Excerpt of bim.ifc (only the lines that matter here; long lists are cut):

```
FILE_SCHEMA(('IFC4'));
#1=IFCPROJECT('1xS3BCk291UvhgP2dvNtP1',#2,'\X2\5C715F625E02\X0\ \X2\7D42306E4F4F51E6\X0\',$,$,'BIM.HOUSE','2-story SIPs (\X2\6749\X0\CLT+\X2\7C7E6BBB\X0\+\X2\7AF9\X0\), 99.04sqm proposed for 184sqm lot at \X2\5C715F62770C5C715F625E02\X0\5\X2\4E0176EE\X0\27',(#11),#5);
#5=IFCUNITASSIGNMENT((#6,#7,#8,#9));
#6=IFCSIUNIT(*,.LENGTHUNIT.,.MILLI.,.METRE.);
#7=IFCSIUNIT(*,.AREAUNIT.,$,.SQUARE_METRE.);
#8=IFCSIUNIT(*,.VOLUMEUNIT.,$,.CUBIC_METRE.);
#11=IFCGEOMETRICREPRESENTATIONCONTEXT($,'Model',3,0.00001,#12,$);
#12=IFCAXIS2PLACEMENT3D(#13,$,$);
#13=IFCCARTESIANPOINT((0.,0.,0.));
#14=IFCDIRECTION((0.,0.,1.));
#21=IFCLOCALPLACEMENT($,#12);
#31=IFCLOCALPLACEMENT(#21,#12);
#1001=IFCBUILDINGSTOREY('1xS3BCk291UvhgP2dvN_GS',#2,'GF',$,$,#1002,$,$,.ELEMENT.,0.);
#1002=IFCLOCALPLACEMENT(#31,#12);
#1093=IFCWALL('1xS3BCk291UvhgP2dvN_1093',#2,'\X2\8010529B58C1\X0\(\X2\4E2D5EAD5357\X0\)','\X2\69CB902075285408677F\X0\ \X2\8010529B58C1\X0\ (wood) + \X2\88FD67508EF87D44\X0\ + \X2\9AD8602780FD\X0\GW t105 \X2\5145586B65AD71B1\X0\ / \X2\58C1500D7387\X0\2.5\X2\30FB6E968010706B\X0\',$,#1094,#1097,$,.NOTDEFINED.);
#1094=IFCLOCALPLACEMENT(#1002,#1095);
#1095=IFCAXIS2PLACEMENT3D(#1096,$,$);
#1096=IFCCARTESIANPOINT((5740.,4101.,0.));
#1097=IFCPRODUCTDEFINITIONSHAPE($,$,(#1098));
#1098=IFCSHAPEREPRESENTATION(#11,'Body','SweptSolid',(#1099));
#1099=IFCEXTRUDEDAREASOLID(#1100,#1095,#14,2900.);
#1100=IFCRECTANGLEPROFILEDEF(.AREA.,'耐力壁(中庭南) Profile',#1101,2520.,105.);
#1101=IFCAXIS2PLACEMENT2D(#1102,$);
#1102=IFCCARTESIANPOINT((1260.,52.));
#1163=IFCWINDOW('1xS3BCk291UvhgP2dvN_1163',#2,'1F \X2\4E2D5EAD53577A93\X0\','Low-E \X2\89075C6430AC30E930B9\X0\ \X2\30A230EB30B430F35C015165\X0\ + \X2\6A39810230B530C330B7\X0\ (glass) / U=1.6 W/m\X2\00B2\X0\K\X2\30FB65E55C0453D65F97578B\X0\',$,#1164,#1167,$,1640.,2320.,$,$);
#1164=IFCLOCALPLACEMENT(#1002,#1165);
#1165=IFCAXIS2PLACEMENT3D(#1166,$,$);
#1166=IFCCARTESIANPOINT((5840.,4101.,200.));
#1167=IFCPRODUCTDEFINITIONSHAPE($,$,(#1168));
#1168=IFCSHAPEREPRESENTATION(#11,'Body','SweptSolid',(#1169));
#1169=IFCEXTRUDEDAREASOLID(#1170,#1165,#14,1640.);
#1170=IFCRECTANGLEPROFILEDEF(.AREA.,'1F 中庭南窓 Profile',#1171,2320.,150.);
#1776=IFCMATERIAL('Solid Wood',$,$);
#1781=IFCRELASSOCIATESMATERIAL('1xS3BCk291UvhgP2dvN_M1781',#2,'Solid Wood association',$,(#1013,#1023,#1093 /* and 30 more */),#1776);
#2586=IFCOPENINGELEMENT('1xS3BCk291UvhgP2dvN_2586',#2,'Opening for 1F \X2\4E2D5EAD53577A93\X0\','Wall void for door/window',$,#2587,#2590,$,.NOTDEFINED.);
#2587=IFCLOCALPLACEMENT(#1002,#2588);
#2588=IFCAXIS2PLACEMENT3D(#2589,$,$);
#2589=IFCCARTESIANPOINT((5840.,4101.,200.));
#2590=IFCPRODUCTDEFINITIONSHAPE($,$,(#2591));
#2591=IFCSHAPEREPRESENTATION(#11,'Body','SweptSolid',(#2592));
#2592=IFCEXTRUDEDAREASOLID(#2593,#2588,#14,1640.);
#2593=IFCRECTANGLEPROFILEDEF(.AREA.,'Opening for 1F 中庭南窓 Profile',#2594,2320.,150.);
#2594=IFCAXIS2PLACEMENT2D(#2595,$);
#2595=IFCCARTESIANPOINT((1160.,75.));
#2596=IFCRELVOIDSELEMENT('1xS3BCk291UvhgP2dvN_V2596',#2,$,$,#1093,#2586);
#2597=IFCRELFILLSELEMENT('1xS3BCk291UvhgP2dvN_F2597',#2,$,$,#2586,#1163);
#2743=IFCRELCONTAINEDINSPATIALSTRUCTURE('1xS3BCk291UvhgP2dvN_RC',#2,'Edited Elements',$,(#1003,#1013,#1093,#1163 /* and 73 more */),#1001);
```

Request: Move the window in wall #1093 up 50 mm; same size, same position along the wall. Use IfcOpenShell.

```python
import numpy as np
import ifcopenshell
import ifcopenshell.api.geometry
import ifcopenshell.util.placement
import ifcopenshell.util.unit

model = ifcopenshell.open("bim.ifc")
unit_scale = ifcopenshell.util.unit.calculate_unit_scale(model)

window = model.by_guid("1xS3BCk291UvhgP2dvN_1163")
opening = window.FillsVoids[0].RelatingOpeningElement
dz = 0.05 / unit_scale

shift = np.array([0.0, 0.0, dz])
# The window is not placed relative to its opening, so move both.
for product in (opening, window):
    matrix = ifcopenshell.util.placement.get_local_placement(product.ObjectPlacement)
    matrix[:3, 3] += shift
    ifcopenshell.api.geometry.edit_object_placement(model, product=product, matrix=matrix, is_si=False)

print(f"moved by {dz * unit_scale:+.3f} m")

model.write("bim-out.ifc")
```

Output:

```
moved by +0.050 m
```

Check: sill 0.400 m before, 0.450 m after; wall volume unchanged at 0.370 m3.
